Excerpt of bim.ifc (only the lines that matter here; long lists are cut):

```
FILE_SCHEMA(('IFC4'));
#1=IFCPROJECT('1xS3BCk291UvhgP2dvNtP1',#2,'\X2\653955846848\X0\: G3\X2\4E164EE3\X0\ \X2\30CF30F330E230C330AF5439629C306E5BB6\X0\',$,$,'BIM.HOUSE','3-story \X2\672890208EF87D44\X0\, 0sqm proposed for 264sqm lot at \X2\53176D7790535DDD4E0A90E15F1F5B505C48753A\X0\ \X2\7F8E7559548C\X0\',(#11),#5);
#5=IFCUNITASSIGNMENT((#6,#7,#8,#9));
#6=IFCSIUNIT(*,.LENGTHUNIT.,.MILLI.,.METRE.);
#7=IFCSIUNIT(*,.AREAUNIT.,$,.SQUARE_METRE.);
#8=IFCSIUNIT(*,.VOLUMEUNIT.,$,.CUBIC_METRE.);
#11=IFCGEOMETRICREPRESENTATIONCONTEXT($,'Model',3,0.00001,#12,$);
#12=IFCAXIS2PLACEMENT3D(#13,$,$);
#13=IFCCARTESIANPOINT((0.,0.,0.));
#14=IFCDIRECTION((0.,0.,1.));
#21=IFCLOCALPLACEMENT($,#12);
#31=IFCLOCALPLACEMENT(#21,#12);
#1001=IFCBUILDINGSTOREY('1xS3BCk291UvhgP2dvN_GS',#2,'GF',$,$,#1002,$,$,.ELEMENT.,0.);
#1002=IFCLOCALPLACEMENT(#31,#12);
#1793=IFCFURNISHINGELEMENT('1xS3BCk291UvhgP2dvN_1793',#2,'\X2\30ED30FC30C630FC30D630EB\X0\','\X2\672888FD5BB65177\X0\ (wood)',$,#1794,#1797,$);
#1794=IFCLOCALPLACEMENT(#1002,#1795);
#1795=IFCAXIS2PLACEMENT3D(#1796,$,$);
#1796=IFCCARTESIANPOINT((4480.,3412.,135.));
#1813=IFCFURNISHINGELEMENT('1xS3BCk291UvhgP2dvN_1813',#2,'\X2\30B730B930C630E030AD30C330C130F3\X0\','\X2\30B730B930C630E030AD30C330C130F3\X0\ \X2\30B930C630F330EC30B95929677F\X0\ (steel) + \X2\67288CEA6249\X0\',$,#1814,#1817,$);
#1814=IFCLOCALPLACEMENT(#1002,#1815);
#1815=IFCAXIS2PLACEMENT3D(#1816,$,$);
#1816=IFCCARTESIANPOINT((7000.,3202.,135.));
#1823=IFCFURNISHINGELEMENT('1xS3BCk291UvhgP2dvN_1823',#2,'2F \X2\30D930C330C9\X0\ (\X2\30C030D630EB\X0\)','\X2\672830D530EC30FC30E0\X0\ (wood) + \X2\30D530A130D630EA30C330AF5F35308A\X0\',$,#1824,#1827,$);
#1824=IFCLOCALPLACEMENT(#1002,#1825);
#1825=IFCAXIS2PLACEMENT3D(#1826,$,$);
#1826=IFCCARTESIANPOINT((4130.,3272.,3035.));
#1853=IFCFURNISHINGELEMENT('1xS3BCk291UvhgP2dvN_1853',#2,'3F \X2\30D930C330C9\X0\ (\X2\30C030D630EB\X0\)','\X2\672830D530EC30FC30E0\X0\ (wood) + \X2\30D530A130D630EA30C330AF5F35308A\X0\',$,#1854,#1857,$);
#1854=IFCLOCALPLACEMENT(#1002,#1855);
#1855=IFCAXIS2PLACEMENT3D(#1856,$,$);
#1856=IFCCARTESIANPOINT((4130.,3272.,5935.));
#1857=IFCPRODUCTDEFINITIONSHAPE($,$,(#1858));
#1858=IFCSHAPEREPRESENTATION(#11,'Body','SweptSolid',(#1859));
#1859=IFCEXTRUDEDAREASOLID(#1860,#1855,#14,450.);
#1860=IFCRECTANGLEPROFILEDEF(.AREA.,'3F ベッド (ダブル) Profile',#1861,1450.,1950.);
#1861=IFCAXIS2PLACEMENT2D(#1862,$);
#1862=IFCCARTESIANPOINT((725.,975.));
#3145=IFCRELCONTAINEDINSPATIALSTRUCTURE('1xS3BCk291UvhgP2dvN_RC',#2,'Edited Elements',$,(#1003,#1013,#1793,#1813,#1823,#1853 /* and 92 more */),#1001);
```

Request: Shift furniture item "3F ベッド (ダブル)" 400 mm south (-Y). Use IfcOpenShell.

```python
import ifcopenshell
import ifcopenshell.api.geometry
import ifcopenshell.util.placement
import ifcopenshell.util.unit

model = ifcopenshell.open("bim.ifc")
unit_scale = ifcopenshell.util.unit.calculate_unit_scale(model)

item = model.by_guid("1xS3BCk291UvhgP2dvN_1853")
matrix = ifcopenshell.util.placement.get_local_placement(item.ObjectPlacement)
matrix[1, 3] -= 0.4 / unit_scale
ifcopenshell.api.geometry.edit_object_placement(model, product=item, matrix=matrix, is_si=False)

print(ifcopenshell.util.placement.get_local_placement(item.ObjectPlacement).round(3) + 0.0)

model.write("bim_v2.ifc")
```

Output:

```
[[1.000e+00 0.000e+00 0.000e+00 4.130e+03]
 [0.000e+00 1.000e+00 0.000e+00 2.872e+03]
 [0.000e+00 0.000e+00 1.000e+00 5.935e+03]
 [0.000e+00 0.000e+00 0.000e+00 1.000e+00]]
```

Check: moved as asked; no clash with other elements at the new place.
